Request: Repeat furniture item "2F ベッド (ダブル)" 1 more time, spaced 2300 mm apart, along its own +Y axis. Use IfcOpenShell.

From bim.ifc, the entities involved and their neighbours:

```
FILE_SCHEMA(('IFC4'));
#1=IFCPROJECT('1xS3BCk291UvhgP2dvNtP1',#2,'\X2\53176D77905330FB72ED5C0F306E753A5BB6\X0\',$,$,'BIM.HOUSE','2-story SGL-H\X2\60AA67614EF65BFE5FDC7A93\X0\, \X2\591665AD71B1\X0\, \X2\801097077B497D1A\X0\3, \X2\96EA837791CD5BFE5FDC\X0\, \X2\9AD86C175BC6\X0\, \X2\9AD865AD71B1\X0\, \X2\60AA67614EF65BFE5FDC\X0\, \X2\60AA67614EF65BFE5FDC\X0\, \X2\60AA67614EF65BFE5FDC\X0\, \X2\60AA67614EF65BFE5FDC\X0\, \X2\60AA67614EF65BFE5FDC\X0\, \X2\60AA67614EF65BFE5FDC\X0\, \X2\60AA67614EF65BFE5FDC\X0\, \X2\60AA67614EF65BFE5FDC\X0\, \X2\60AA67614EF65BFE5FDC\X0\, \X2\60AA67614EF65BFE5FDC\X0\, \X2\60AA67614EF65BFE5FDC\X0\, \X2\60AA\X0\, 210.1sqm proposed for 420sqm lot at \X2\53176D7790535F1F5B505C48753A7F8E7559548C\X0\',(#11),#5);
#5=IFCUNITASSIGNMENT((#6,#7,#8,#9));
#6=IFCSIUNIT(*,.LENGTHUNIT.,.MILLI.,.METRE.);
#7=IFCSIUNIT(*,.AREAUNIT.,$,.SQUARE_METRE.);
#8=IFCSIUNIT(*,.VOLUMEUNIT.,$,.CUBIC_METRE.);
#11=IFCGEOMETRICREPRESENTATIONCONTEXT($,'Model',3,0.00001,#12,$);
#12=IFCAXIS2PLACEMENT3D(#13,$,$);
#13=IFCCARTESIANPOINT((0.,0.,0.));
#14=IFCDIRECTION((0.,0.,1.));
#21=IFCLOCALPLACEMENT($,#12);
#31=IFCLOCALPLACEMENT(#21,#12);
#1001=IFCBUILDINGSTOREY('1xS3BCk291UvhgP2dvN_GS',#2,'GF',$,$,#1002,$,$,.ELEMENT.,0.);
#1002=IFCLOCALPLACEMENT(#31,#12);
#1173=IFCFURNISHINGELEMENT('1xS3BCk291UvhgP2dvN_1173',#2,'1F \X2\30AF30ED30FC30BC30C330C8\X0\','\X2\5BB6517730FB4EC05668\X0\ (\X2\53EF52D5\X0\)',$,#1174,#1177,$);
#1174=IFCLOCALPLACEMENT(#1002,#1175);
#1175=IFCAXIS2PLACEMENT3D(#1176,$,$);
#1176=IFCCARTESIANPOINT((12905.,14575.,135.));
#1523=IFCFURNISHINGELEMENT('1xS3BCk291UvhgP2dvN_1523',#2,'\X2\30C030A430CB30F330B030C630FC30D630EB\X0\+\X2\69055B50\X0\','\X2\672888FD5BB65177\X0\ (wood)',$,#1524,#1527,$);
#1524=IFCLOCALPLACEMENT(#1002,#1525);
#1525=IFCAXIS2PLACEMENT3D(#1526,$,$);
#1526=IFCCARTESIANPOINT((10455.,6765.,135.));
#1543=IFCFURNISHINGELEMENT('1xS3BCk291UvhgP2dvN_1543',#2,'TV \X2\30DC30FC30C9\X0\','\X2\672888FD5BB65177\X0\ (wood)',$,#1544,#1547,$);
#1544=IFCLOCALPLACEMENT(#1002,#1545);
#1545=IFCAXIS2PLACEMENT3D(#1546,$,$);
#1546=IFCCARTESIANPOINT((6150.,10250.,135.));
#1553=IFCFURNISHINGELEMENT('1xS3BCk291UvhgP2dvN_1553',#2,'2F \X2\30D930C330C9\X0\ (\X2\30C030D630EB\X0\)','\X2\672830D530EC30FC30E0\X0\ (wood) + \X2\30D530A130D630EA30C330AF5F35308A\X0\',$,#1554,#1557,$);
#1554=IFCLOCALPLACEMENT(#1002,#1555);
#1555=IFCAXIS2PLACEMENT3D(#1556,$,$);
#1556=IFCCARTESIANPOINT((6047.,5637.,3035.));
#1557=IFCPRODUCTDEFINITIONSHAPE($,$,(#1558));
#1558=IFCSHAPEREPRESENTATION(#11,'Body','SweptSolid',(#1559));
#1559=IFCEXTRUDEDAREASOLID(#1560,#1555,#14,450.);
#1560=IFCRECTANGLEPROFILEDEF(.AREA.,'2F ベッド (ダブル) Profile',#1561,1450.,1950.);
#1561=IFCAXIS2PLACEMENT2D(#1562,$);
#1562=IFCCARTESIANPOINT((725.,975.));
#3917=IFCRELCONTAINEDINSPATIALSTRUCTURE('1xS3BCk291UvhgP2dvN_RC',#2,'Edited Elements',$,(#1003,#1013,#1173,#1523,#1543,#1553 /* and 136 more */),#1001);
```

```python
import ifcopenshell
import ifcopenshell.api.geometry
import ifcopenshell.api.root
import ifcopenshell.util.element
import ifcopenshell.util.placement
import ifcopenshell.util.unit

model = ifcopenshell.open("bim.ifc")
unit_scale = ifcopenshell.util.unit.calculate_unit_scale(model)


def reuse_history(source, copy):
    """copy_class also copies each property set's owner history, people and application; keep the originals."""
    for rel in copy.IsDefinedBy:
        if rel.is_a("IfcRelDefinesByProperties") and (history := rel.RelatingPropertyDefinition.OwnerHistory):
            rel.RelatingPropertyDefinition.OwnerHistory = source.OwnerHistory
            ifcopenshell.util.element.remove_deep2(model, history)


source = model.by_guid("1xS3BCk291UvhgP2dvN_1553")
base = ifcopenshell.util.placement.get_local_placement(source.ObjectPlacement)
step = base[:3, 1] * 2.3 / unit_scale

for i in range(1, 2):
    copy = ifcopenshell.api.root.copy_class(model, product=source)
    copy.Representation = ifcopenshell.util.element.copy_deep(
        model, source.Representation, exclude=["IfcGeometricRepresentationContext", "IfcRepresentationMap"]
    )
    reuse_history(source, copy)
    matrix = base.copy()
    matrix[:3, 3] += i * step
    print("added at", matrix[:3, 3].round(3) + 0.0)
    ifcopenshell.api.geometry.edit_object_placement(model, product=copy, matrix=matrix, is_si=False)

model.write("bim_v2.ifc")
```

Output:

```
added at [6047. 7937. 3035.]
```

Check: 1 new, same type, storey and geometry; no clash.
